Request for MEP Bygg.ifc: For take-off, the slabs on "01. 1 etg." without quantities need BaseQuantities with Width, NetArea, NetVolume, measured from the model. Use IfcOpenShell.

First a look at what the model holds.

```python
import ifcopenshell
import ifcopenshell.util.element
import ifcopenshell.util.unit

model = ifcopenshell.open("MEP Bygg.ifc")
print(model.schema)
for unit_type in ("LENGTHUNIT", "AREAUNIT", "VOLUMEUNIT"):
    print(unit_type, ifcopenshell.util.unit.calculate_unit_scale(model, unit_type))
storey = next(s for s in model.by_type("IfcBuildingStorey") if s.Name == "01. 1 etg.")
slabs = [e for e in ifcopenshell.util.element.get_decomposition(storey) if e.is_a("IfcSlab")]
for e in sorted(slabs, key=lambda e: e.id()):
    print(e.id(), e.is_a(), e.Name, list(ifcopenshell.util.element.get_psets(e, qtos_only=True)), sep=" | ")
```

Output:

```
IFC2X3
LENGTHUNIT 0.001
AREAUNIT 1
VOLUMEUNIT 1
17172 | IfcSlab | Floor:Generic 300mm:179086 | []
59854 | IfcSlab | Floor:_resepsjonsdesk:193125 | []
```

```python
import ifcopenshell
import ifcopenshell.api.pset
import ifcopenshell.geom
import ifcopenshell.util.element
import ifcopenshell.util.shape
import ifcopenshell.util.unit

model = ifcopenshell.open("MEP Bygg.ifc")
unit_scale = ifcopenshell.util.unit.calculate_unit_scale(model)
area_scale = ifcopenshell.util.unit.calculate_unit_scale(model, "AREAUNIT")
volume_scale = ifcopenshell.util.unit.calculate_unit_scale(model, "VOLUMEUNIT")
settings = ifcopenshell.geom.settings()

storey = next(s for s in model.by_type("IfcBuildingStorey") if s.Name == "01. 1 etg.")
slabs = [e for e in ifcopenshell.util.element.get_decomposition(storey) if e.is_a("IfcSlab")]

for e in sorted(slabs, key=lambda e: e.id()):
    if ifcopenshell.util.element.get_psets(e, qtos_only=True, should_inherit=False):
        continue
    # Geometry comes back in metres, in the element's own axes.
    shape = ifcopenshell.geom.create_shape(settings, e)
    values = {
        "Width": ifcopenshell.util.shape.get_z(shape.geometry) / unit_scale,
        "NetArea": ifcopenshell.util.shape.get_footprint_area(shape.geometry) / area_scale,
        "NetVolume": ifcopenshell.util.shape.get_volume(shape.geometry) / volume_scale,
    }
    qto = ifcopenshell.api.pset.add_qto(model, product=e, name="BaseQuantities")
    ifcopenshell.api.pset.edit_qto(model, qto=qto, properties=values)
    print(e.id(), {k: round(v, 3) for k, v in values.items()})

model.write("MEP Bygg_edited.ifc")
```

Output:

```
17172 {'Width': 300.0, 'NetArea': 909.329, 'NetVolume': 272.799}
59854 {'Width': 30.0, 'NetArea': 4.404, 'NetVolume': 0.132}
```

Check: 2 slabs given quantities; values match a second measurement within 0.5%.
